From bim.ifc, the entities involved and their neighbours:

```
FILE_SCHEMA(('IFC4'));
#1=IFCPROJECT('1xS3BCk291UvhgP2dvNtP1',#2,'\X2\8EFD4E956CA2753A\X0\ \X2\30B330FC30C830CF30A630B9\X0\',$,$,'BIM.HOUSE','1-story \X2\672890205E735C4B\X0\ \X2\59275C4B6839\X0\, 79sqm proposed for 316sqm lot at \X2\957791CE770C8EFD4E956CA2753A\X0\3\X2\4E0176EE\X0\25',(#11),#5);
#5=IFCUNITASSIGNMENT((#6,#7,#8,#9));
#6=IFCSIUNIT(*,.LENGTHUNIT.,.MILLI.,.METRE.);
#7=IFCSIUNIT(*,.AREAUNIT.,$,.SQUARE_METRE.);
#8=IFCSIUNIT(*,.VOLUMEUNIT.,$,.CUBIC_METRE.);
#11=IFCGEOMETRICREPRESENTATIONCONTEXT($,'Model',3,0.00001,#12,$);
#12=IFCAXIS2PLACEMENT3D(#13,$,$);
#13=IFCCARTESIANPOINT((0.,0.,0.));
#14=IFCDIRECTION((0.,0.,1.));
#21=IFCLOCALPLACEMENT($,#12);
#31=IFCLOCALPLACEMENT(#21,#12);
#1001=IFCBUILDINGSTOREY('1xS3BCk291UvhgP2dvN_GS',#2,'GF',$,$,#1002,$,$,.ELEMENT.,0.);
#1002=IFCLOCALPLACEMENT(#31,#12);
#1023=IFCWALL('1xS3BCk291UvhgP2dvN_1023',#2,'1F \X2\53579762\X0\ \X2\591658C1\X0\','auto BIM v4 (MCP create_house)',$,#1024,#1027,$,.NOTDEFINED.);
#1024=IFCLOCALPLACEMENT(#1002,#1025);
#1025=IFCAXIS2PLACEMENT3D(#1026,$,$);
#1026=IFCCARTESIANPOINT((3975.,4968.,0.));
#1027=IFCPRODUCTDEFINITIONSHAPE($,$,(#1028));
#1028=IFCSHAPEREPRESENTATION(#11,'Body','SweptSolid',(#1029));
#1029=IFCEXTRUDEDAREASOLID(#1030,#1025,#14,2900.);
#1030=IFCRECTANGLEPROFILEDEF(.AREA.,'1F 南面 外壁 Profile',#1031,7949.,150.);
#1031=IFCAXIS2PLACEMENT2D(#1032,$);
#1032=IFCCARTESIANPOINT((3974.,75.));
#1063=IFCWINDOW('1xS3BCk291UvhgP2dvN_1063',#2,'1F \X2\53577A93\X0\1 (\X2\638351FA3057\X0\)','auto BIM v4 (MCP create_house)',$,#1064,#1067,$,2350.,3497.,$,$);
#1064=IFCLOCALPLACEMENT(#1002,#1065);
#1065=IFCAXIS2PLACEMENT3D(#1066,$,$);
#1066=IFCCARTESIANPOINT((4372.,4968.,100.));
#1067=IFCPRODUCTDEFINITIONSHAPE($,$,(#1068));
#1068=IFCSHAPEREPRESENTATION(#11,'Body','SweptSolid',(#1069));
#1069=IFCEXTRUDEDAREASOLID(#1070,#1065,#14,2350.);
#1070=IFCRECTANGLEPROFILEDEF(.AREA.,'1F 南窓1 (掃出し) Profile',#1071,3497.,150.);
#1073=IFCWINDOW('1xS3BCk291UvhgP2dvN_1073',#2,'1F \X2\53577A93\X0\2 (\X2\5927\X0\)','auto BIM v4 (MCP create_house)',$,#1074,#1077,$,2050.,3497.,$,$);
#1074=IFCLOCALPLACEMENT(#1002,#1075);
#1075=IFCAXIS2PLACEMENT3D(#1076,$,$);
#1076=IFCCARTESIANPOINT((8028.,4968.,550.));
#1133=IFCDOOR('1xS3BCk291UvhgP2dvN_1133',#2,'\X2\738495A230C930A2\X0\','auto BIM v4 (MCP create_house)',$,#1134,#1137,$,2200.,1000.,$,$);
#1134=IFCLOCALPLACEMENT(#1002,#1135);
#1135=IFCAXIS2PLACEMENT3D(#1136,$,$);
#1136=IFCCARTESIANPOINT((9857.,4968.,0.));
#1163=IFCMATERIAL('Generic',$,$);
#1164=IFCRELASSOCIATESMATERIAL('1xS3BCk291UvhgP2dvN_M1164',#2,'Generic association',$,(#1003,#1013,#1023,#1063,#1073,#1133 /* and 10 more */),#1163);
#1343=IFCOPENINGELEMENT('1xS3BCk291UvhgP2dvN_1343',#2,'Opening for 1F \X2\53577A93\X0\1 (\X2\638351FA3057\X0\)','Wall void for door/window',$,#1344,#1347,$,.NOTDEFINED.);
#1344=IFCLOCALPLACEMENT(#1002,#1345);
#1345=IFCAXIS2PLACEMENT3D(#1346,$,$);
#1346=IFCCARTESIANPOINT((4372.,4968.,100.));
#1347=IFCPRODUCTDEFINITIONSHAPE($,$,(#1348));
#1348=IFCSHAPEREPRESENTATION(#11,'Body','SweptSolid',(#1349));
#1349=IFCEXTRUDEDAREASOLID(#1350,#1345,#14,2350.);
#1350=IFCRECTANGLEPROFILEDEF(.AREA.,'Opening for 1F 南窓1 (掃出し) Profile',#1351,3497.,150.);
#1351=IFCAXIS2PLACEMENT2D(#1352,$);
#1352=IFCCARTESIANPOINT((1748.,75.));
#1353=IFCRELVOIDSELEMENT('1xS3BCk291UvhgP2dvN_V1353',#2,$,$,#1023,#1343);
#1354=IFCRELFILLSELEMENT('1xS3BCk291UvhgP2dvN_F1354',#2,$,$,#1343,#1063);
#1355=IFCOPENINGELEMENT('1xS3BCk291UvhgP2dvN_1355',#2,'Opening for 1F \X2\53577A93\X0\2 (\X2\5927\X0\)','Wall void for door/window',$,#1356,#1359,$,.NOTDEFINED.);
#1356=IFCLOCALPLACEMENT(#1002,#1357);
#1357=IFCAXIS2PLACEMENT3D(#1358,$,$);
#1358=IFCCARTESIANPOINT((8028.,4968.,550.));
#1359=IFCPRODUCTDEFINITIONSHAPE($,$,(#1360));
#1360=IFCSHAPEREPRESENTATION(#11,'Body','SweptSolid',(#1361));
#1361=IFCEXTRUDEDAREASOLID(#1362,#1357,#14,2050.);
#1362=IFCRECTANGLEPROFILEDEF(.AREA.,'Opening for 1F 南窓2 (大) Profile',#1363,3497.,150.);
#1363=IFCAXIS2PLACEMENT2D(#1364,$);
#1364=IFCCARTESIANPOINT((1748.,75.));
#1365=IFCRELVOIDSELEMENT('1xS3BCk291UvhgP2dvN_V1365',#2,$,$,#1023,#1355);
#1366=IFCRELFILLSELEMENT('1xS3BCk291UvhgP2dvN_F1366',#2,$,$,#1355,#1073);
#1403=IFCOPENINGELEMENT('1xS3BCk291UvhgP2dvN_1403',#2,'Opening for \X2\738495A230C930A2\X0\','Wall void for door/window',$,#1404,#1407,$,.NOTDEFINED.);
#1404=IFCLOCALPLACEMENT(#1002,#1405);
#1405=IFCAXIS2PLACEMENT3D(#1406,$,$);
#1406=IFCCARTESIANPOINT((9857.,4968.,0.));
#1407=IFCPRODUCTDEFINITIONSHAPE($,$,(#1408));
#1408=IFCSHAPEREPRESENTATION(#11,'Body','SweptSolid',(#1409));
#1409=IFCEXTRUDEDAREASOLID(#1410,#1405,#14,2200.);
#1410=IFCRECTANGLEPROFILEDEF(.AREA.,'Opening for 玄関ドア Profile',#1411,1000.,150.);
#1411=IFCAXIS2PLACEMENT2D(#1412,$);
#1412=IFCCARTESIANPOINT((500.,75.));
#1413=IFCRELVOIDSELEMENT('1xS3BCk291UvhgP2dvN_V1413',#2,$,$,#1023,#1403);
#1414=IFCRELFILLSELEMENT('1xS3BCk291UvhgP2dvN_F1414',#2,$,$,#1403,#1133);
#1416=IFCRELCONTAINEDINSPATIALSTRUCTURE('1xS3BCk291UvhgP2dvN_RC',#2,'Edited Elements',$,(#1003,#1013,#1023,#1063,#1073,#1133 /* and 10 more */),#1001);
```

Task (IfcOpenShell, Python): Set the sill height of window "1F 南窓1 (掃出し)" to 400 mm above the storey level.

```python
import numpy as np
import ifcopenshell
import ifcopenshell.api.geometry
import ifcopenshell.geom
import ifcopenshell.util.element
import ifcopenshell.util.placement
import ifcopenshell.util.shape
import ifcopenshell.util.unit

model = ifcopenshell.open("bim.ifc")
unit_scale = ifcopenshell.util.unit.calculate_unit_scale(model)

window = model.by_guid("1xS3BCk291UvhgP2dvN_1063")
opening = window.FillsVoids[0].RelatingOpeningElement
storey = ifcopenshell.util.element.get_container(window, ifc_class="IfcBuildingStorey")
level = ifcopenshell.util.placement.get_local_placement(storey.ObjectPlacement)[2, 3]

# The opening's origin need not be at the sill, so measure its lowest point.
shape = ifcopenshell.geom.create_shape(ifcopenshell.geom.settings(), opening)
bottom = ifcopenshell.util.shape.get_shape_bottom_elevation(shape, shape.geometry) / unit_scale
dz = level + 0.4 / unit_scale - bottom

shift = np.array([0.0, 0.0, dz])
# The window is not placed relative to its opening, so move both.
for product in (opening, window):
    matrix = ifcopenshell.util.placement.get_local_placement(product.ObjectPlacement)
    matrix[:3, 3] += shift
    ifcopenshell.api.geometry.edit_object_placement(model, product=product, matrix=matrix, is_si=False)

print(f"moved by {dz * unit_scale:+.3f} m")

model.write("bim-out.ifc")
```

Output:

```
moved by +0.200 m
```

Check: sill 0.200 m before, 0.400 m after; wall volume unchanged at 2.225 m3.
